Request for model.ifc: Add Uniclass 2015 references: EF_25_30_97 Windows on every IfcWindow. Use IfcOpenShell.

First a look at what the model holds.

```python
import ifcopenshell

model = ifcopenshell.open("model.ifc")
print(model.schema)
print("classifications:", [c.Name for c in model.by_type("IfcClassification")])
for ifc_class in ("IfcDoor", "IfcRoof", "IfcStair", "IfcWall", "IfcWindow"):
    print(ifc_class, len(model.by_type(ifc_class)))
```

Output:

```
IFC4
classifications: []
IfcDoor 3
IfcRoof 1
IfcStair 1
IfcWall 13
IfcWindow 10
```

```python
import ifcopenshell
import ifcopenshell.api.classification

model = ifcopenshell.open("model.ifc")

system = ifcopenshell.api.classification.add_classification(model, classification="Uniclass 2015")

codes = {
    "IfcWindow": ("EF_25_30_97", "Windows"),
}
for ifc_class, (code, name) in codes.items():
    products = model.by_type(ifc_class)
    ifcopenshell.api.classification.add_reference(
        model, products=products, classification=system, identification=code, name=name
    )
    print(code, len(products))

model.write("model-out.ifc")
```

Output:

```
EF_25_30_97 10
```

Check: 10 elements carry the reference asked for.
